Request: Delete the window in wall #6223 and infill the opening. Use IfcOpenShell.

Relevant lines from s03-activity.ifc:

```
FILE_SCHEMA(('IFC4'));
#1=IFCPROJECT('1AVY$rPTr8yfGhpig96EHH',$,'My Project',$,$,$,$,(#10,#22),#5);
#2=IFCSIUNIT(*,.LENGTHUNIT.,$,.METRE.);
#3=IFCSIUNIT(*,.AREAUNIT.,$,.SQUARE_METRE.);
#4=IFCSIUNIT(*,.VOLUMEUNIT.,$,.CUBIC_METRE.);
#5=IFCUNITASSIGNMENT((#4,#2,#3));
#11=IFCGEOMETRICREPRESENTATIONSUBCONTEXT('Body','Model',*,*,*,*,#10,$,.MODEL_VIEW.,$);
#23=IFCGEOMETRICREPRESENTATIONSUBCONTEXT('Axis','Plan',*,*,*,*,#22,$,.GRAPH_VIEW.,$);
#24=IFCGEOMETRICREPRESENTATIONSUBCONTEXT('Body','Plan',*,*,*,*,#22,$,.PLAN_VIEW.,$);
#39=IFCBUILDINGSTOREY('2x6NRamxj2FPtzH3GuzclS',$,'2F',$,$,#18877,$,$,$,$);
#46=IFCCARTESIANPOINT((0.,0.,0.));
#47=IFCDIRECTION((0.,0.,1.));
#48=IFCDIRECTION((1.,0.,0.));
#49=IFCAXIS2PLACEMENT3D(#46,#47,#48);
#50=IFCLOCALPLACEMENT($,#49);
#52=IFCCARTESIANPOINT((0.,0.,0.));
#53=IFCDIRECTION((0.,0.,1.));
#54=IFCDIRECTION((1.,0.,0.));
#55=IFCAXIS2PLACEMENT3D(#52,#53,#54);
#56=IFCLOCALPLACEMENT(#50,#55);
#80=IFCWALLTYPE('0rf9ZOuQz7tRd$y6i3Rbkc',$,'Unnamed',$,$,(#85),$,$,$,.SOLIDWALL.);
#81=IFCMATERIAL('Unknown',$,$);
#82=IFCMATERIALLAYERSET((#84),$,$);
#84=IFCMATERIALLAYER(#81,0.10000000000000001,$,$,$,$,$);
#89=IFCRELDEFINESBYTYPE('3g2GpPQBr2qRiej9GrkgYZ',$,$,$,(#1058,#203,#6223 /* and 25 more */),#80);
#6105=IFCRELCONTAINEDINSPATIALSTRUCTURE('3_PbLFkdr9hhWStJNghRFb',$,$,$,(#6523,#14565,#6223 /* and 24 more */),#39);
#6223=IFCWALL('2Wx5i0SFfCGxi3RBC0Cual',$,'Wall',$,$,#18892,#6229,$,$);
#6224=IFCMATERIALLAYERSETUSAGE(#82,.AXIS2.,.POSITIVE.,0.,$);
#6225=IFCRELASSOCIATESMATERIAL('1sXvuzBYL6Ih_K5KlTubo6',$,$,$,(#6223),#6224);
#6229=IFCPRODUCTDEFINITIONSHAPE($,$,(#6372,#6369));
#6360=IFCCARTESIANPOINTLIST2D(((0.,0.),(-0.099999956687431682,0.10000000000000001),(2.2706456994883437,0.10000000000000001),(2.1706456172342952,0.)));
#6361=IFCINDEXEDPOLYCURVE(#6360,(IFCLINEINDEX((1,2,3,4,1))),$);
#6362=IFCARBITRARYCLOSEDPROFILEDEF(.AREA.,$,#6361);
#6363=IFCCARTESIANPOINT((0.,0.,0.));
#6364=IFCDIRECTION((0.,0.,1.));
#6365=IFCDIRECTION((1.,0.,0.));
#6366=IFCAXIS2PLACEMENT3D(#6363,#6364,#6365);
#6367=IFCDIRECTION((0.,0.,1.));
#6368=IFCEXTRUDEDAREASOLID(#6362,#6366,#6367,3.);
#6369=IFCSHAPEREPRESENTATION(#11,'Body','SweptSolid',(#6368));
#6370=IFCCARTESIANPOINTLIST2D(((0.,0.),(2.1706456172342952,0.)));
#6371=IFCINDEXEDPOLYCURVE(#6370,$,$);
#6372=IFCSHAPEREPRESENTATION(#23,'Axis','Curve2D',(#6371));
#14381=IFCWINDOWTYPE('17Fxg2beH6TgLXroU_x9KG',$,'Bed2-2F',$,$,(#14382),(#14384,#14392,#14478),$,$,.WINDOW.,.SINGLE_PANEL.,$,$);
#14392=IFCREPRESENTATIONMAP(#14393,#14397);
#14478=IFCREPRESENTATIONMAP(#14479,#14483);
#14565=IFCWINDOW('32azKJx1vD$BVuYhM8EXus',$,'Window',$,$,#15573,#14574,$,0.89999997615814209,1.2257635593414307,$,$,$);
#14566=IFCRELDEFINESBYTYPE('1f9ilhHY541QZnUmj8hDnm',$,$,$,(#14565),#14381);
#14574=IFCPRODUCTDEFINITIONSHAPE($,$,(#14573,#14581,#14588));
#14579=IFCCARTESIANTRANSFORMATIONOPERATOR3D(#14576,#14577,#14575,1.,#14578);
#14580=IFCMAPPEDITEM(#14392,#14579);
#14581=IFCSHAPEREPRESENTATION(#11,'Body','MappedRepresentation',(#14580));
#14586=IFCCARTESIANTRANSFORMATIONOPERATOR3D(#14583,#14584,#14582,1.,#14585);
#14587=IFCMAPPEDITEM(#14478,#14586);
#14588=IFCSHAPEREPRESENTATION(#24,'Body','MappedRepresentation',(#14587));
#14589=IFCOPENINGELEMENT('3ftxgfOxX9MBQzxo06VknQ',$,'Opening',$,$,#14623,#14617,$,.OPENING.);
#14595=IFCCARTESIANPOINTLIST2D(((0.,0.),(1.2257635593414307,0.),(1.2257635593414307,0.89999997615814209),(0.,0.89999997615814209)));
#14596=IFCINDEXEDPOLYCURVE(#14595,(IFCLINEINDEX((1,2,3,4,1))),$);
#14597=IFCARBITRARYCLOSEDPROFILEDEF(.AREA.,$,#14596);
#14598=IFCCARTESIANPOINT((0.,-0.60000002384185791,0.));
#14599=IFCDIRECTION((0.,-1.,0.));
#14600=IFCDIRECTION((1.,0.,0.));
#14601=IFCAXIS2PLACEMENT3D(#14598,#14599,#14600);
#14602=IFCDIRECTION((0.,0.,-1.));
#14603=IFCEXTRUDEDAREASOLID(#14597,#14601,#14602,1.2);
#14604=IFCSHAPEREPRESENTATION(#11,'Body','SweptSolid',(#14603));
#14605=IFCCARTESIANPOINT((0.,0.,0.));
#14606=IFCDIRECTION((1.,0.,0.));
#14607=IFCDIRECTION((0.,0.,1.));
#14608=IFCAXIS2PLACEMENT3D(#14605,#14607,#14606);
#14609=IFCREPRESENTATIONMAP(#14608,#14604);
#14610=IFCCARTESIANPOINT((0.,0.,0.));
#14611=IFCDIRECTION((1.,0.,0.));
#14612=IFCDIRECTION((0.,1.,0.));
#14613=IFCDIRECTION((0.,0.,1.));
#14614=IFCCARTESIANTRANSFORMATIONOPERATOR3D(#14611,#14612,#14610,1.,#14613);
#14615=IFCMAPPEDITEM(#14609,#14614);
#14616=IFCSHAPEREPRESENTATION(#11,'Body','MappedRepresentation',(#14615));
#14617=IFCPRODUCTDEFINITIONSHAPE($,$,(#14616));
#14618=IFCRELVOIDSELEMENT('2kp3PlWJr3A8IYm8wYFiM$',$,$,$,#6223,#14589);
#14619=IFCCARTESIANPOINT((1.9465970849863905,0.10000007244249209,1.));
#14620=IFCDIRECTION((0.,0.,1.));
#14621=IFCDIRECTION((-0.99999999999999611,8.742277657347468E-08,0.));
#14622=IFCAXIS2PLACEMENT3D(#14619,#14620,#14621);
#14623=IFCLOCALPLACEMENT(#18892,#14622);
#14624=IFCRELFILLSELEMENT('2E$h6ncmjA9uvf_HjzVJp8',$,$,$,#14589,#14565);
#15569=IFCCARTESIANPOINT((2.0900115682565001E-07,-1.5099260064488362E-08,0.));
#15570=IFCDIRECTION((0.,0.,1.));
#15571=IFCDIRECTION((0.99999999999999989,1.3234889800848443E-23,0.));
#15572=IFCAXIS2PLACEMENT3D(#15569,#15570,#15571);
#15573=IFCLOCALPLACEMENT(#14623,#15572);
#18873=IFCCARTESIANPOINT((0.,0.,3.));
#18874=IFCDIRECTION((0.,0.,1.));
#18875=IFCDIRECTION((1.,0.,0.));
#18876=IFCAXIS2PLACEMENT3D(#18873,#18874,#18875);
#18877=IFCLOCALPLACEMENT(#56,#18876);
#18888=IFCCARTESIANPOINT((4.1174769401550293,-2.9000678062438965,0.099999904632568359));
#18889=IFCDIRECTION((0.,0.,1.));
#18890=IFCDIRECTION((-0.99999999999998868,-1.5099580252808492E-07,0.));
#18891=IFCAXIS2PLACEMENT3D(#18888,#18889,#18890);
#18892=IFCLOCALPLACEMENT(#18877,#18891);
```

```python
import ifcopenshell
import ifcopenshell.api.feature
import ifcopenshell.api.root
import ifcopenshell.geom
import ifcopenshell.util.shape

model = ifcopenshell.open("s03-activity.ifc")
settings = ifcopenshell.geom.settings()


def volume(element):
    """Net volume in cubic metres, openings subtracted."""
    shape = ifcopenshell.geom.create_shape(settings, element)
    return ifcopenshell.util.shape.get_volume(shape.geometry)


window = model.by_guid("32azKJx1vD$BVuYhM8EXus")
opening = window.FillsVoids[0].RelatingOpeningElement
wall = opening.VoidsElements[0].RelatingBuildingElement
before = volume(wall)

ifcopenshell.api.root.remove_product(model, product=window)
ifcopenshell.api.feature.remove_feature(model, feature=opening)

after = volume(wall)

print(f"wall volume {before:.3f} -> {after:.3f} m3")

model.write("s03-activity_updated.ifc")
```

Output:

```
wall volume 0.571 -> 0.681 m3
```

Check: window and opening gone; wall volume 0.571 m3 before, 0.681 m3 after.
